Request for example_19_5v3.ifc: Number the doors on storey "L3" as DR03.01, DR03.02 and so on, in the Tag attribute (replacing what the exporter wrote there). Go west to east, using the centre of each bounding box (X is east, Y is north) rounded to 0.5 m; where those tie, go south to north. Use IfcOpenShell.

First a look at what the model holds.

```python
import ifcopenshell
import ifcopenshell.util.element
import ifcopenshell.util.placement

model = ifcopenshell.open("example_19_5v3.ifc")
print(model.schema)
storey = next(s for s in model.by_type("IfcBuildingStorey") if s.Name == "L3")
doors = [e for e in ifcopenshell.util.element.get_decomposition(storey) if e.is_a("IfcDoor")]
for e in sorted(doors, key=lambda e: e.id()):
    origin = ifcopenshell.util.placement.get_local_placement(e.ObjectPlacement)[:3, 3]
    print(e.id(), e.Tag, e.Name, origin.round(2) + 0.0, sep=" | ")
```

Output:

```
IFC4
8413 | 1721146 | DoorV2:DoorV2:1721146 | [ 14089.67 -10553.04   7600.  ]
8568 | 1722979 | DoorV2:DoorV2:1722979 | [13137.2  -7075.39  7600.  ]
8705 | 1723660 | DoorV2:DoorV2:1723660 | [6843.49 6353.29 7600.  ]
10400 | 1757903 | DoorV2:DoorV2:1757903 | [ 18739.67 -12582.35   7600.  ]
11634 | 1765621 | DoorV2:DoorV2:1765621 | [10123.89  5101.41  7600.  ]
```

```python
import ifcopenshell
import ifcopenshell.geom
import ifcopenshell.util.element
import ifcopenshell.util.shape

model = ifcopenshell.open("example_19_5v3.ifc")
settings = ifcopenshell.geom.settings()
settings.set("use-world-coords", True)


def centre(element):
    shape = ifcopenshell.geom.create_shape(settings, element)
    return ifcopenshell.util.shape.get_bbox_centroid(shape.geometry)


storey = next(s for s in model.by_type("IfcBuildingStorey") if s.Name == "L3")
doors = [e for e in ifcopenshell.util.element.get_decomposition(storey) if e.is_a("IfcDoor")]

# Insertion points can sit at a corner or the storey origin, so sort by the geometry (in metres).
centres = {e: centre(e) for e in doors}
doors.sort(key=lambda e: (round(centres[e][0] / 0.5), centres[e][1]))

for i, e in enumerate(doors, start=1):
    number = f"DR03.{i:02d}"
    e.Tag = number
    print(e.id(), number)

model.write("example_19_5v3-out.ifc")
```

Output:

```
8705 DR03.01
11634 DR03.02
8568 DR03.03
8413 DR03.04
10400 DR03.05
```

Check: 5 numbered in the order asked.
